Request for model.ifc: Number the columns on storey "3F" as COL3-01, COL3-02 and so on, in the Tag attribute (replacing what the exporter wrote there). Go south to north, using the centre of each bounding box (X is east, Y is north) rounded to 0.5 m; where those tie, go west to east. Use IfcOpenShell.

First a look at what the model holds.

```python
import ifcopenshell
import ifcopenshell.util.element
import ifcopenshell.util.placement

model = ifcopenshell.open("model.ifc")
print(model.schema)
storey = next(s for s in model.by_type("IfcBuildingStorey") if s.Name == "3F")
columns = [e for e in ifcopenshell.util.element.get_decomposition(storey) if e.is_a("IfcColumn")]
for e in sorted(columns, key=lambda e: e.id()):
    origin = ifcopenshell.util.placement.get_local_placement(e.ObjectPlacement)[:3, 3]
    print(e.id(), e.Tag, e.Name, origin.round(2) + 0.0, sep=" | ")
```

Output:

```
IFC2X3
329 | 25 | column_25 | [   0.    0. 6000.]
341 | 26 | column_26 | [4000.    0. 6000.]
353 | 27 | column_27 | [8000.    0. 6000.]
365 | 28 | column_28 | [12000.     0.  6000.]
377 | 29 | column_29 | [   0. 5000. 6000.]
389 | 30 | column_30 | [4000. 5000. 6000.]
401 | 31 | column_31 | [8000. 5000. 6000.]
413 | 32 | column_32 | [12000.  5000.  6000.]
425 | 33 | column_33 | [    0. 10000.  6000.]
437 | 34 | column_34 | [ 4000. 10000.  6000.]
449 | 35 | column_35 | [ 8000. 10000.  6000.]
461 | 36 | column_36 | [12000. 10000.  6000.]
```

```python
import ifcopenshell
import ifcopenshell.geom
import ifcopenshell.util.element
import ifcopenshell.util.shape

model = ifcopenshell.open("model.ifc")
settings = ifcopenshell.geom.settings()
settings.set("use-world-coords", True)


def centre(element):
    shape = ifcopenshell.geom.create_shape(settings, element)
    return ifcopenshell.util.shape.get_bbox_centroid(shape.geometry)


storey = next(s for s in model.by_type("IfcBuildingStorey") if s.Name == "3F")
columns = [e for e in ifcopenshell.util.element.get_decomposition(storey) if e.is_a("IfcColumn")]

# Insertion points can sit at a corner or the storey origin, so sort by the geometry (in metres).
centres = {e: centre(e) for e in columns}
columns.sort(key=lambda e: (round(centres[e][1] / 0.5), centres[e][0]))

for i, e in enumerate(columns, start=1):
    number = f"COL3-{i:02d}"
    e.Tag = number
    print(e.id(), number)

model.write("model_v2.ifc")
```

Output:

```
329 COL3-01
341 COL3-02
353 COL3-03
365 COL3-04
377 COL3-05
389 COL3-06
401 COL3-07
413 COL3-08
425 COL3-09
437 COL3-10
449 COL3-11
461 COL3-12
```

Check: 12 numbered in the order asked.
